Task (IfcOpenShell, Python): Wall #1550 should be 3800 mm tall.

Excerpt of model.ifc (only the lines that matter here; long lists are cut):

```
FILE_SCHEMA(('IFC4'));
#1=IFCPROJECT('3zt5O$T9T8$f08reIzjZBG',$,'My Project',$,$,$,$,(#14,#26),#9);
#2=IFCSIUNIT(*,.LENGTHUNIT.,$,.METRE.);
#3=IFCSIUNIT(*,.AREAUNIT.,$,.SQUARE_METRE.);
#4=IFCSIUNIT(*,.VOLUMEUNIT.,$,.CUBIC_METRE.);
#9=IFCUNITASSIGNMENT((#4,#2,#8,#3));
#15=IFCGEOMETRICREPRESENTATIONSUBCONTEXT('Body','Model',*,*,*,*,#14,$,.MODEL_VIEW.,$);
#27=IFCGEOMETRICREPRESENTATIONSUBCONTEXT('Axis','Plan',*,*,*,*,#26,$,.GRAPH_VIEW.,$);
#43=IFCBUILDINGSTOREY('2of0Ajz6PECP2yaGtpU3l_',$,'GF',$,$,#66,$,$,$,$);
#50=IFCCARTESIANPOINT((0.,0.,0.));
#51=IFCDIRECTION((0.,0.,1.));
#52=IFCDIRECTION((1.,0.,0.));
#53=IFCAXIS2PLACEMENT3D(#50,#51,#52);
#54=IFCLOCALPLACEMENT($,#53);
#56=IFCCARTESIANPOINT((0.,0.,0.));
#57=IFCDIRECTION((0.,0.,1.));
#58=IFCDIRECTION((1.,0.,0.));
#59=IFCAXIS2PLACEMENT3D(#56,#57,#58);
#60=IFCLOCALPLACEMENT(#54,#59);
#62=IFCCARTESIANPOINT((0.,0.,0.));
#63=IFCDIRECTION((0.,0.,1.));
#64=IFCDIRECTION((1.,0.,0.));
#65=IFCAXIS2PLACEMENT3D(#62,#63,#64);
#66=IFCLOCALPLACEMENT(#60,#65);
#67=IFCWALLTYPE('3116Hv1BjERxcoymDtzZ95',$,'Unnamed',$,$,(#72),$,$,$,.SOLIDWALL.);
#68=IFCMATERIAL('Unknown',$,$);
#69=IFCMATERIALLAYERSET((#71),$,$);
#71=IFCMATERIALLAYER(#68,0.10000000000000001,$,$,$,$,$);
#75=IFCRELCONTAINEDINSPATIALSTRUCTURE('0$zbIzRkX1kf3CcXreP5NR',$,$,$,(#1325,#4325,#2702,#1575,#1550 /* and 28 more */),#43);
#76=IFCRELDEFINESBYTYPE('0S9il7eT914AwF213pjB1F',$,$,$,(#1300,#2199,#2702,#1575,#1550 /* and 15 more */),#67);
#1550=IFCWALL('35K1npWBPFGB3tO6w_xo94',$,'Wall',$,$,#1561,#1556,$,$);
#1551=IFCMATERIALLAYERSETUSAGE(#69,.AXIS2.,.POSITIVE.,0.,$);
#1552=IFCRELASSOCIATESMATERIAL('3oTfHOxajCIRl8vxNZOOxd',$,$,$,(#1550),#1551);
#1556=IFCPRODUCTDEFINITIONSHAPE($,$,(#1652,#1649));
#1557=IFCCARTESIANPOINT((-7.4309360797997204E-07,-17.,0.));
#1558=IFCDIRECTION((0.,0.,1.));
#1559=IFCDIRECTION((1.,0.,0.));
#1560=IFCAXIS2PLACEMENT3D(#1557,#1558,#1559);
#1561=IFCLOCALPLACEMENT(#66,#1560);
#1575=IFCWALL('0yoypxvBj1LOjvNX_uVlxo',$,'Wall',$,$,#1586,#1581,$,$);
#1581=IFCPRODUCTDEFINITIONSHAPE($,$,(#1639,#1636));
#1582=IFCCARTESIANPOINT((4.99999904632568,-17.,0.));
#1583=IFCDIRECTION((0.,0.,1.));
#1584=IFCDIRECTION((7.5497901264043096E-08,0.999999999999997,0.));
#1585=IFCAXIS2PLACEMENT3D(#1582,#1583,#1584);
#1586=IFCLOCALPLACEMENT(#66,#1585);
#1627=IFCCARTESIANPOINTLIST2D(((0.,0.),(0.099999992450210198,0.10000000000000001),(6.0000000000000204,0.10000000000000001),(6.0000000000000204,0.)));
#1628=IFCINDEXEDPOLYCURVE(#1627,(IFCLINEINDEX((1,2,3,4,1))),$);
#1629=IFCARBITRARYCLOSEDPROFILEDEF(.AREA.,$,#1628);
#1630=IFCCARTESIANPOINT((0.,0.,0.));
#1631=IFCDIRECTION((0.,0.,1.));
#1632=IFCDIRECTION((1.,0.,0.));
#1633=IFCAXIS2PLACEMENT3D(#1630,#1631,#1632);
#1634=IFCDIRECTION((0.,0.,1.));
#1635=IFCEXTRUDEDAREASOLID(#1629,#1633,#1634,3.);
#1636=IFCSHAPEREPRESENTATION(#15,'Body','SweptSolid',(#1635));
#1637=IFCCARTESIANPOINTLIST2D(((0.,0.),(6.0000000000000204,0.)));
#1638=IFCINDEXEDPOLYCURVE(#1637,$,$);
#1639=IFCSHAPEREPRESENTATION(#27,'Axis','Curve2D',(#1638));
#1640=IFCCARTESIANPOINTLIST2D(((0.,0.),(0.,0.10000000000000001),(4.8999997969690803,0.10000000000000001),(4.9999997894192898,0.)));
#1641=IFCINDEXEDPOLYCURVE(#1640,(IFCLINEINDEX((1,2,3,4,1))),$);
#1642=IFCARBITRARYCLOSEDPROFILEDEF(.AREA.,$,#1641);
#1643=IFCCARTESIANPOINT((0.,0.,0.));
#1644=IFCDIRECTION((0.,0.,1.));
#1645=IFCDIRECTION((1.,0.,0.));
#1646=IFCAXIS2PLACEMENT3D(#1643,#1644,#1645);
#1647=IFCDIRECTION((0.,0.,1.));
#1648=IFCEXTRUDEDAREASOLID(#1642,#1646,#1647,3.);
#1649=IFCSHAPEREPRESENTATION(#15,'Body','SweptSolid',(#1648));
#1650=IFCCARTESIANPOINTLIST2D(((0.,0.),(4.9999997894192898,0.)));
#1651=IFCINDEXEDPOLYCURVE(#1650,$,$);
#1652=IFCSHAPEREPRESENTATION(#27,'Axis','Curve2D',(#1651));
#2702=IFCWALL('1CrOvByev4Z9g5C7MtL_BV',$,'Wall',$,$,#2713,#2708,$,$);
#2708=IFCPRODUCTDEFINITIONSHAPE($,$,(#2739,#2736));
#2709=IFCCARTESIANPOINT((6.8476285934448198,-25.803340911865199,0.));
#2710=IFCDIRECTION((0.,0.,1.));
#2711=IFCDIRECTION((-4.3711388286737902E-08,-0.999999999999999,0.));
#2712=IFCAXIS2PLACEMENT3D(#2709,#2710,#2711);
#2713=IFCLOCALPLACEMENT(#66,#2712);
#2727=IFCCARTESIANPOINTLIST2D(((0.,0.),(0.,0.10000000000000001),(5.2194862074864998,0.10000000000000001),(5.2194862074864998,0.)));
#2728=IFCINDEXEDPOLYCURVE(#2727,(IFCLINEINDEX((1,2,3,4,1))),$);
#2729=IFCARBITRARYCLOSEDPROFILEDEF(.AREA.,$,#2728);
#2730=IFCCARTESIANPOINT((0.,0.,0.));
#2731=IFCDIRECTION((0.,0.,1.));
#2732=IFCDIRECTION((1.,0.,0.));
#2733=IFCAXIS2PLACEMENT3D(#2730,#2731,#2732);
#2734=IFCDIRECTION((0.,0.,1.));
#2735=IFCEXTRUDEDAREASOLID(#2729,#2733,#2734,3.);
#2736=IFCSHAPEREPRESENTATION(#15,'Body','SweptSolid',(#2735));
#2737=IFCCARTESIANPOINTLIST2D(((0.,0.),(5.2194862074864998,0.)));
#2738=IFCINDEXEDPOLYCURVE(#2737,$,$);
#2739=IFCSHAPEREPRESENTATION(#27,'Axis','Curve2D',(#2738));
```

```python
import ifcopenshell
import ifcopenshell.geom
import ifcopenshell.util.representation
import ifcopenshell.util.shape
import ifcopenshell.util.unit

model = ifcopenshell.open("model.ifc")
unit_scale = ifcopenshell.util.unit.calculate_unit_scale(model)
settings = ifcopenshell.geom.settings()


def volume(element):
    """Net volume in cubic metres, openings subtracted."""
    shape = ifcopenshell.geom.create_shape(settings, element)
    return ifcopenshell.util.shape.get_volume(shape.geometry)


wall = model.by_guid("35K1npWBPFGB3tO6w_xo94")
before = volume(wall)

body = ifcopenshell.util.representation.get_representation(wall, "Model", "Body")
solid = body.Items[0]
old_height = solid.Depth
solid.Depth = 3.8 / unit_scale
after = volume(wall)

print(f"height {old_height:g} -> {solid.Depth:g}, volume {before:.3f} -> {after:.3f} m3")

model.write("model-out.ifc")
```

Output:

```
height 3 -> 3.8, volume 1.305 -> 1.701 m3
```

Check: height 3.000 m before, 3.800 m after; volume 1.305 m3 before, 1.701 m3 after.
